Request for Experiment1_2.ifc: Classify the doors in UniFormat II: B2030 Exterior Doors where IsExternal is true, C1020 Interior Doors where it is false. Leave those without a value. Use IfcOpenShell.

First a look at what the model holds.

```python
import ifcopenshell
import ifcopenshell.util.element

model = ifcopenshell.open("Experiment1_2.ifc")
print(model.schema)
print("classifications:", [c.Name for c in model.by_type("IfcClassification")])
values = [ifcopenshell.util.element.get_pset(e, "Pset_DoorCommon", "IsExternal") for e in model.by_type("IfcDoor")]
for value in (True, False, None):
    print("IsExternal", value, values.count(value))
```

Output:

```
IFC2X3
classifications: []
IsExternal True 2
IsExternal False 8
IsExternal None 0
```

```python
import ifcopenshell
import ifcopenshell.api.classification
import ifcopenshell.util.element

model = ifcopenshell.open("Experiment1_2.ifc")

# IFC2X3 requires Source and Edition and has no link from the project to the system.
system = model.create_entity("IfcClassification", Source="ASTM", Edition="E1557", Name="UniFormat II")

doors = model.by_type("IfcDoor")
external = {e: ifcopenshell.util.element.get_pset(e, "Pset_DoorCommon", "IsExternal") for e in doors}
for flag, code, name in ((True, "B2030", "Exterior Doors"), (False, "C1020", "Interior Doors")):
    products = [e for e in doors if external[e] is flag]
    ifcopenshell.api.classification.add_reference(
        model, products=products, classification=system, identification=code, name=name
    )
    print(code, len(products))

model.write("Experiment1_2_updated.ifc")
```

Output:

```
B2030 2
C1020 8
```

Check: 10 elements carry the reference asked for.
